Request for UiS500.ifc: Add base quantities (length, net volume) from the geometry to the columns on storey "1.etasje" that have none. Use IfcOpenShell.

First a look at what the model holds.

```python
import ifcopenshell
import ifcopenshell.util.element
import ifcopenshell.util.unit

model = ifcopenshell.open("UiS500.ifc")
print(model.schema)
for unit_type in ("LENGTHUNIT", "AREAUNIT", "VOLUMEUNIT"):
    print(unit_type, ifcopenshell.util.unit.calculate_unit_scale(model, unit_type))
storey = next(s for s in model.by_type("IfcBuildingStorey") if s.Name == "1.etasje")
columns = [e for e in ifcopenshell.util.element.get_decomposition(storey) if e.is_a("IfcColumn")]
for e in sorted(columns, key=lambda e: e.id()):
    print(e.id(), e.is_a(), e.Name, list(ifcopenshell.util.element.get_psets(e, qtos_only=True)), sep=" | ")
```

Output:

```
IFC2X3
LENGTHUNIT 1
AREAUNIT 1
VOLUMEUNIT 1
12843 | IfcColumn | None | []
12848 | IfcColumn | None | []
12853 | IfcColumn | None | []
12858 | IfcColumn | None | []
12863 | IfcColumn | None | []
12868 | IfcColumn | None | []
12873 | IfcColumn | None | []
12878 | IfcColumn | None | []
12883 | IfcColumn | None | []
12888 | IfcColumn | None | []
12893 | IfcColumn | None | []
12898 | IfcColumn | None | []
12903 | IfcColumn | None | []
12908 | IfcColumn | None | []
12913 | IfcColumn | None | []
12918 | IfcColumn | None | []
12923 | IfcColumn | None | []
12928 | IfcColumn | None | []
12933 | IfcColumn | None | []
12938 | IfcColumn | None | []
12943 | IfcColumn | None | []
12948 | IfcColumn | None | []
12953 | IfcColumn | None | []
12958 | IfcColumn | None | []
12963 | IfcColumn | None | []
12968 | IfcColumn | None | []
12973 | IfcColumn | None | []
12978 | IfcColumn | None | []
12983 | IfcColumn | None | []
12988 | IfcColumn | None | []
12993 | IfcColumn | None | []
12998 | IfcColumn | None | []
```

```python
import ifcopenshell
import ifcopenshell.api.pset
import ifcopenshell.geom
import ifcopenshell.util.element
import ifcopenshell.util.shape
import ifcopenshell.util.unit

model = ifcopenshell.open("UiS500.ifc")
unit_scale = ifcopenshell.util.unit.calculate_unit_scale(model)
volume_scale = ifcopenshell.util.unit.calculate_unit_scale(model, "VOLUMEUNIT")
settings = ifcopenshell.geom.settings()

storey = next(s for s in model.by_type("IfcBuildingStorey") if s.Name == "1.etasje")
columns = [e for e in ifcopenshell.util.element.get_decomposition(storey) if e.is_a("IfcColumn")]

for e in sorted(columns, key=lambda e: e.id()):
    if ifcopenshell.util.element.get_psets(e, qtos_only=True, should_inherit=False):
        continue
    # Geometry comes back in metres, in the element's own axes.
    shape = ifcopenshell.geom.create_shape(settings, e)
    values = {
        "Length": ifcopenshell.util.shape.get_z(shape.geometry) / unit_scale,
        "NetVolume": ifcopenshell.util.shape.get_volume(shape.geometry) / volume_scale,
    }
    qto = ifcopenshell.api.pset.add_qto(model, product=e, name="BaseQuantities")
    ifcopenshell.api.pset.edit_qto(model, qto=qto, properties=values)
    print(e.id(), {k: round(v, 3) for k, v in values.items()})

model.write("UiS500_edited.ifc")
```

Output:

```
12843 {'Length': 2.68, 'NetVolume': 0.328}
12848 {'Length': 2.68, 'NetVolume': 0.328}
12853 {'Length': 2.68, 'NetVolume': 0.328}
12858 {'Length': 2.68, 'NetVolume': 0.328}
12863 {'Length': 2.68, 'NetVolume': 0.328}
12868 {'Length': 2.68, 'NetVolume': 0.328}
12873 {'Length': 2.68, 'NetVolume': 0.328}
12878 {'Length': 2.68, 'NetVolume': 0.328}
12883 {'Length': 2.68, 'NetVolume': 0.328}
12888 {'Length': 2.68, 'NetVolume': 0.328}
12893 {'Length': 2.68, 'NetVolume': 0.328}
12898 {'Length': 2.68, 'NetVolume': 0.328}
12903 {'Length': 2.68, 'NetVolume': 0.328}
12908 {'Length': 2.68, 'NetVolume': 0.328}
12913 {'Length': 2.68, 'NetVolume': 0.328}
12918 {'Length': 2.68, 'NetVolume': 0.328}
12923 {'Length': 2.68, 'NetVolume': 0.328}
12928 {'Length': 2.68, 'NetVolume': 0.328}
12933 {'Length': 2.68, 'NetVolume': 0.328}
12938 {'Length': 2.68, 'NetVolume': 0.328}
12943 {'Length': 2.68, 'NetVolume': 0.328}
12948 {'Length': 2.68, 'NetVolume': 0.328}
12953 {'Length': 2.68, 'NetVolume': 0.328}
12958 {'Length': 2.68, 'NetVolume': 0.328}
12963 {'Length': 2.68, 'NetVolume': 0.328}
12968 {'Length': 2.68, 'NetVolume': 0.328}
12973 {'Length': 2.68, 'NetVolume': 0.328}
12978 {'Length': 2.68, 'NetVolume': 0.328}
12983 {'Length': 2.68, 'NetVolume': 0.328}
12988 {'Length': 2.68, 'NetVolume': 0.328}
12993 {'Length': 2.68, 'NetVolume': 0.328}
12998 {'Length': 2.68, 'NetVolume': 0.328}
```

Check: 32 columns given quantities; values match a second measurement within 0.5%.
